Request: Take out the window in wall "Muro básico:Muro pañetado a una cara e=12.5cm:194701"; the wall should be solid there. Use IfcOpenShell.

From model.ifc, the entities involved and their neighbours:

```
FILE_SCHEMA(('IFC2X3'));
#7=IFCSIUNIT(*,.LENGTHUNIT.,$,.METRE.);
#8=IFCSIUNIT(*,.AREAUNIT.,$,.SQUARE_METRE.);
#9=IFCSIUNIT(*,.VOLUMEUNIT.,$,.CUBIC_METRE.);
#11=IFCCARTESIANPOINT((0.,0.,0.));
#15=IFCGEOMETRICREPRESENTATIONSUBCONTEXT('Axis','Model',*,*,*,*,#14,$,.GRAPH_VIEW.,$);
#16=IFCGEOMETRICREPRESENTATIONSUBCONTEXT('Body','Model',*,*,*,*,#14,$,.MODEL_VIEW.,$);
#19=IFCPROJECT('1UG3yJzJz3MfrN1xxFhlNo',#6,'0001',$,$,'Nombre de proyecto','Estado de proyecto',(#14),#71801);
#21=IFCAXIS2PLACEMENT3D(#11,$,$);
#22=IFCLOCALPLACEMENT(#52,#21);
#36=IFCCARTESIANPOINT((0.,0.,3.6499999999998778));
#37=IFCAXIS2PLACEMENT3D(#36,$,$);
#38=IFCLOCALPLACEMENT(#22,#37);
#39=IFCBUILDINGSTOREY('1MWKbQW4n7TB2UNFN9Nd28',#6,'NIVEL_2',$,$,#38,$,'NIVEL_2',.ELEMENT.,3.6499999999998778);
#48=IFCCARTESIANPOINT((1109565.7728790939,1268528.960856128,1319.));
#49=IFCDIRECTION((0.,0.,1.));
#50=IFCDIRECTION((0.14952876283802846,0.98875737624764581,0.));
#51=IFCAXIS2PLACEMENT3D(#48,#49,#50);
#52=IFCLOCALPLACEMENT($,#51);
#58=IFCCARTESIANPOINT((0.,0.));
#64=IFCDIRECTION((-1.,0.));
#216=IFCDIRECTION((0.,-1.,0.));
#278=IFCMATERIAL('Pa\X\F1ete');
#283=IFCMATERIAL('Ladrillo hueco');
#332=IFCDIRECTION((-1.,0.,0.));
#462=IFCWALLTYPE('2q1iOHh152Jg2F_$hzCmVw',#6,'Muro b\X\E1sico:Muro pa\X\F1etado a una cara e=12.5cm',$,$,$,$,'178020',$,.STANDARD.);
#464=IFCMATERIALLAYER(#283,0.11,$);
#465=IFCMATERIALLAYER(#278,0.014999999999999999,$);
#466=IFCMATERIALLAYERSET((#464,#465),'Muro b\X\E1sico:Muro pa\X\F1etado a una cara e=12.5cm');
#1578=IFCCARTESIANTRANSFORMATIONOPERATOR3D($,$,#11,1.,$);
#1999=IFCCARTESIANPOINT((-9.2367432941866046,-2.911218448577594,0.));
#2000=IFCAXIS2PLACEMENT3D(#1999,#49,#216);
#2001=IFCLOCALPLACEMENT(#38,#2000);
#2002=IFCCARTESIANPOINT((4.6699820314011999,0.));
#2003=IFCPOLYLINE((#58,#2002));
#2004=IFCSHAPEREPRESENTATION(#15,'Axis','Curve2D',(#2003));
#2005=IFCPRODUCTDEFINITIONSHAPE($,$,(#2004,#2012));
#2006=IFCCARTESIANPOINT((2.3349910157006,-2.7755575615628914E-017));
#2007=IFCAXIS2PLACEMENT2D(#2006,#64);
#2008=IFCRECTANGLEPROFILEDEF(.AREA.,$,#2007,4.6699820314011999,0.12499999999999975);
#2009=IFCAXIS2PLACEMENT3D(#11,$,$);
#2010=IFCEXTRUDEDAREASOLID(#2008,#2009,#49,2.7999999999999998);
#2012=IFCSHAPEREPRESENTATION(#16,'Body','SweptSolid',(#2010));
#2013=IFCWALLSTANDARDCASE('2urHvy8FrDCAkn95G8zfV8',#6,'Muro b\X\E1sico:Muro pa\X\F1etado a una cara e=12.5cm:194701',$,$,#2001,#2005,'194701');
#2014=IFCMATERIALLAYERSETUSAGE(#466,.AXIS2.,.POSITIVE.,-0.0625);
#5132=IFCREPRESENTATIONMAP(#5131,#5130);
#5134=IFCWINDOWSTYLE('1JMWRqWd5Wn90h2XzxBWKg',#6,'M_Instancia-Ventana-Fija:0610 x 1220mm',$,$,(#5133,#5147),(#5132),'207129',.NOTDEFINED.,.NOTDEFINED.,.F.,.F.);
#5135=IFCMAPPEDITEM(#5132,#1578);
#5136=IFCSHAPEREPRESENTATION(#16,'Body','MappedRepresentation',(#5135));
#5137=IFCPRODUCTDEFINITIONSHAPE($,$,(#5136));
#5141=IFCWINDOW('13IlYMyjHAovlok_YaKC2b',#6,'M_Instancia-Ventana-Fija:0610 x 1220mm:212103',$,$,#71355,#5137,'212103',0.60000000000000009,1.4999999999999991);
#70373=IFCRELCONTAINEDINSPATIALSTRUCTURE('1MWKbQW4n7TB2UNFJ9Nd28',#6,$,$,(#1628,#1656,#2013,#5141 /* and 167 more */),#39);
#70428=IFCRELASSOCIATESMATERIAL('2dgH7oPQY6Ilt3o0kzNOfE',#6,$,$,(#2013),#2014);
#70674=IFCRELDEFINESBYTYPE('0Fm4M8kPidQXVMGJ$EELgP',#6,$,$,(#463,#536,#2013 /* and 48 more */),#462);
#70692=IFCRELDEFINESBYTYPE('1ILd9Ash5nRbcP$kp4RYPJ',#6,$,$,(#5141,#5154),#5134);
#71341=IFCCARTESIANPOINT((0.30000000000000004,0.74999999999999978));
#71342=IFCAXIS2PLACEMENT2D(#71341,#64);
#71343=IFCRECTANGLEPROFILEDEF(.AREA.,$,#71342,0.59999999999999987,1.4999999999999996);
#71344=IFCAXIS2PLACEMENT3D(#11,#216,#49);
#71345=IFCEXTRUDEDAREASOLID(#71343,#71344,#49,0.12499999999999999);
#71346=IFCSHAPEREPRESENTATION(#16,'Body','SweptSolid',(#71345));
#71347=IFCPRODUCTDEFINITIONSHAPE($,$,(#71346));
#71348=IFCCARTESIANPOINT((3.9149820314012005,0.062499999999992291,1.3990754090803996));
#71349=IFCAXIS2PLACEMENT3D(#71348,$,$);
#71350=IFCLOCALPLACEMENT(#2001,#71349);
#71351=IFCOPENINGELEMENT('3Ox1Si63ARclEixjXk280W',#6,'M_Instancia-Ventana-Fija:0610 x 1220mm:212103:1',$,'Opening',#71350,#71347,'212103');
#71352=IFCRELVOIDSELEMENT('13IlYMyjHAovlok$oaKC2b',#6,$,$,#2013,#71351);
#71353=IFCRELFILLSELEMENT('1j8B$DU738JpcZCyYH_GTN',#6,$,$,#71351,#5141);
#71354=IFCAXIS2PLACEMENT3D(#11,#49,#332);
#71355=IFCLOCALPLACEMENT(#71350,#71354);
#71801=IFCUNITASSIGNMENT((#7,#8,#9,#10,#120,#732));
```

```python
import ifcopenshell
import ifcopenshell.api.feature
import ifcopenshell.api.root
import ifcopenshell.geom
import ifcopenshell.util.shape

model = ifcopenshell.open("model.ifc")
settings = ifcopenshell.geom.settings()


def volume(element):
    """Net volume in cubic metres, openings subtracted."""
    shape = ifcopenshell.geom.create_shape(settings, element)
    return ifcopenshell.util.shape.get_volume(shape.geometry)


window = model.by_guid("13IlYMyjHAovlok_YaKC2b")
opening = window.FillsVoids[0].RelatingOpeningElement
wall = opening.VoidsElements[0].RelatingBuildingElement
before = volume(wall)

ifcopenshell.api.root.remove_product(model, product=window)
ifcopenshell.api.feature.remove_feature(model, feature=opening)

after = volume(wall)

print(f"wall volume {before:.3f} -> {after:.3f} m3")

model.write("model_edited.ifc")
```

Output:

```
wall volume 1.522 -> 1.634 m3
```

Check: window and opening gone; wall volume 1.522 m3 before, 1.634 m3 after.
